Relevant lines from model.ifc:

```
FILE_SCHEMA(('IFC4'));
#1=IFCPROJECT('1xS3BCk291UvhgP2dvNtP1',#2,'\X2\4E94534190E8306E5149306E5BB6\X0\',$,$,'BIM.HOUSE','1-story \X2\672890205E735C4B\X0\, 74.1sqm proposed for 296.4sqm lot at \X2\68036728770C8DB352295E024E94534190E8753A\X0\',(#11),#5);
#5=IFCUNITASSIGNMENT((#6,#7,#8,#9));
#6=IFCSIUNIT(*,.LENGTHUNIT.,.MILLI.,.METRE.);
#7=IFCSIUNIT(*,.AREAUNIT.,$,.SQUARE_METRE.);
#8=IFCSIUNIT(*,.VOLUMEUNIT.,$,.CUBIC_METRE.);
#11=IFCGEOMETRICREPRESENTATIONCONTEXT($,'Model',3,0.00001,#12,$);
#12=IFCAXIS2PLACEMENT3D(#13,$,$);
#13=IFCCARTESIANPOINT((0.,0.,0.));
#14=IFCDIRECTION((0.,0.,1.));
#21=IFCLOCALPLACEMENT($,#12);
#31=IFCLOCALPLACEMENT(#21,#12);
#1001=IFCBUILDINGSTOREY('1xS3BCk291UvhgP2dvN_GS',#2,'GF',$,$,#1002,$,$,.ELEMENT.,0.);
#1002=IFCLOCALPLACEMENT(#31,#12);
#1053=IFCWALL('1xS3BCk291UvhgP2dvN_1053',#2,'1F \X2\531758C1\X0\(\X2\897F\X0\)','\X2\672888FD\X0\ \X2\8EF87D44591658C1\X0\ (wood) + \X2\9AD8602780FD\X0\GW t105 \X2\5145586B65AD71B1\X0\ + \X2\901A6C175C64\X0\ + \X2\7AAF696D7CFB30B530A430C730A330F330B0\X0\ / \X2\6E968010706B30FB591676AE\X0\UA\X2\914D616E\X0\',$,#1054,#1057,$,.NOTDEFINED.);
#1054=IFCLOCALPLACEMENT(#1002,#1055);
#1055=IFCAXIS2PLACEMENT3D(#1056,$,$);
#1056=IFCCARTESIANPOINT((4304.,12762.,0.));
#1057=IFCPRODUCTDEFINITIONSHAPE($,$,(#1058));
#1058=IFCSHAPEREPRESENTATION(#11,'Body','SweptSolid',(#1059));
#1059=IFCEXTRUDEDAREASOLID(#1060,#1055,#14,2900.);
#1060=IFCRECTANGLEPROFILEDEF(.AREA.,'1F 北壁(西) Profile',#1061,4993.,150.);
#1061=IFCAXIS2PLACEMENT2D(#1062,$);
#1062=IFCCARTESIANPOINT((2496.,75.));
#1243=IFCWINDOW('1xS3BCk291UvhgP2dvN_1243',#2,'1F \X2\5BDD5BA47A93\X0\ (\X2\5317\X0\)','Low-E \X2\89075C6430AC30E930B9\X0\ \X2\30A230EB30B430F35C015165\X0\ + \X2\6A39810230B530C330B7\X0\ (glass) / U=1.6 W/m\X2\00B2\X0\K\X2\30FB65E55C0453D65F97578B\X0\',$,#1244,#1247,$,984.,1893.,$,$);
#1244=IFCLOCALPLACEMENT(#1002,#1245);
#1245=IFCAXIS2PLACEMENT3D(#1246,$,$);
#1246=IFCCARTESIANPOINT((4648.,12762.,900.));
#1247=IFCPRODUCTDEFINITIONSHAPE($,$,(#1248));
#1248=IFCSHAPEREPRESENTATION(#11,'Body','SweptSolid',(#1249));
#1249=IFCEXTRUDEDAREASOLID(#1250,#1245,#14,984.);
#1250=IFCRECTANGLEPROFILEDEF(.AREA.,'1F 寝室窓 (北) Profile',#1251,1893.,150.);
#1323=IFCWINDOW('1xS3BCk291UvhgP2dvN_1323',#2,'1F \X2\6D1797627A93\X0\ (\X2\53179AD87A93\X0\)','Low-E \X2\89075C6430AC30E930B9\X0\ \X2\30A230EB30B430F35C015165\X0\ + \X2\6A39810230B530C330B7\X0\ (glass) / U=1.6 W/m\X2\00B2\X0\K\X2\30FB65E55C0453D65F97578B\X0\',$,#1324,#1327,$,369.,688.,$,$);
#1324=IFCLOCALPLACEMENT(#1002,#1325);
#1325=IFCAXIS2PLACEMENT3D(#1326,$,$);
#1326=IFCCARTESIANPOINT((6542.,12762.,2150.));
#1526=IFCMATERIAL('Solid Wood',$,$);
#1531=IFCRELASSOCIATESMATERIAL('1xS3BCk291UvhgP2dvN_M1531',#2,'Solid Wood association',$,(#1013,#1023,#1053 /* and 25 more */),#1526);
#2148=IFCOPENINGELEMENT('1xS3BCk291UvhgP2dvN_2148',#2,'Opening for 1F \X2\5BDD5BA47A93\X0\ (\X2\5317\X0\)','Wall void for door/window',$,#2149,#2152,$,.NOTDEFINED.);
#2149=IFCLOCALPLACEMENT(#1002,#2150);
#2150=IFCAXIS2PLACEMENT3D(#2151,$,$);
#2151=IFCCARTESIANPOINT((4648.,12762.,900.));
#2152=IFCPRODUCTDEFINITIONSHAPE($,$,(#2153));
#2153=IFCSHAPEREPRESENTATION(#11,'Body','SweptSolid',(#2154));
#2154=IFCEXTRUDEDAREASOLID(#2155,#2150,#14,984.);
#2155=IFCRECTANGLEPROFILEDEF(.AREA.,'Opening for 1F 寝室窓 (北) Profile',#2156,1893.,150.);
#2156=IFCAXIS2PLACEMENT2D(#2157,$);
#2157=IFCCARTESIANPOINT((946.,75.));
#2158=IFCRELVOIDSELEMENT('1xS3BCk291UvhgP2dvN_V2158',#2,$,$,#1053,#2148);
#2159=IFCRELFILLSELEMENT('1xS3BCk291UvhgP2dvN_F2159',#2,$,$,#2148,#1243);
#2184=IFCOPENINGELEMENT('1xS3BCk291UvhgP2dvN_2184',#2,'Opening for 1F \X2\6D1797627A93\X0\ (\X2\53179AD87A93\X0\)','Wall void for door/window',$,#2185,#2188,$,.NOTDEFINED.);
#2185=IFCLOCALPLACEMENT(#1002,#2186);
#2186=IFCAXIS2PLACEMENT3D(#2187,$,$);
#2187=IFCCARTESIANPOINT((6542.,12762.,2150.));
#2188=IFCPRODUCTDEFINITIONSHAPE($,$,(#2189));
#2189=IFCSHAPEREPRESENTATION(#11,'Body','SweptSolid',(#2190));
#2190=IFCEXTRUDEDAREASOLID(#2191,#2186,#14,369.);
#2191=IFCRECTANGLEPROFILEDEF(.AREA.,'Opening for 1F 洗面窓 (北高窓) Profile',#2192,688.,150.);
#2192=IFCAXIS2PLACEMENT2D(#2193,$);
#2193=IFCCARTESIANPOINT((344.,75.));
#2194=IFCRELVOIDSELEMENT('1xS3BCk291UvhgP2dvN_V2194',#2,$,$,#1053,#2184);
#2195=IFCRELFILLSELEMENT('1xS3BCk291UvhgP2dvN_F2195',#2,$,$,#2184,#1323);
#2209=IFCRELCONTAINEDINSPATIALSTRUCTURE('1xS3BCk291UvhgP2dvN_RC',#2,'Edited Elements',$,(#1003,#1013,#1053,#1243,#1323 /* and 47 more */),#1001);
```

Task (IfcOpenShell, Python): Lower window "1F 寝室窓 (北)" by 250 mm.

```python
import numpy as np
import ifcopenshell
import ifcopenshell.api.geometry
import ifcopenshell.util.placement
import ifcopenshell.util.unit

model = ifcopenshell.open("model.ifc")
unit_scale = ifcopenshell.util.unit.calculate_unit_scale(model)

window = model.by_guid("1xS3BCk291UvhgP2dvN_1243")
opening = window.FillsVoids[0].RelatingOpeningElement
dz = -0.25 / unit_scale

shift = np.array([0.0, 0.0, dz])
# The window is not placed relative to its opening, so move both.
for product in (opening, window):
    matrix = ifcopenshell.util.placement.get_local_placement(product.ObjectPlacement)
    matrix[:3, 3] += shift
    ifcopenshell.api.geometry.edit_object_placement(model, product=product, matrix=matrix, is_si=False)

print(f"moved by {dz * unit_scale:+.3f} m")

model.write("model_v2.ifc")
```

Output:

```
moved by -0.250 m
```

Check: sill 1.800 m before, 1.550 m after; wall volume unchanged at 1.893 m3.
